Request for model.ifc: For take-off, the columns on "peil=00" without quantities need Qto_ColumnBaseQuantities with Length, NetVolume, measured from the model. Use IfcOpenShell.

First a look at what the model holds.

```python
import ifcopenshell
import ifcopenshell.util.element
import ifcopenshell.util.unit

model = ifcopenshell.open("model.ifc")
print(model.schema)
for unit_type in ("LENGTHUNIT", "AREAUNIT", "VOLUMEUNIT"):
    print(unit_type, ifcopenshell.util.unit.calculate_unit_scale(model, unit_type))
storey = next(s for s in model.by_type("IfcBuildingStorey") if s.Name == "peil=00")
columns = [e for e in ifcopenshell.util.element.get_decomposition(storey) if e.is_a("IfcColumn")]
for e in sorted(columns, key=lambda e: e.id()):
    print(e.id(), e.is_a(), e.Name, list(ifcopenshell.util.element.get_psets(e, qtos_only=True)), sep=" | ")
```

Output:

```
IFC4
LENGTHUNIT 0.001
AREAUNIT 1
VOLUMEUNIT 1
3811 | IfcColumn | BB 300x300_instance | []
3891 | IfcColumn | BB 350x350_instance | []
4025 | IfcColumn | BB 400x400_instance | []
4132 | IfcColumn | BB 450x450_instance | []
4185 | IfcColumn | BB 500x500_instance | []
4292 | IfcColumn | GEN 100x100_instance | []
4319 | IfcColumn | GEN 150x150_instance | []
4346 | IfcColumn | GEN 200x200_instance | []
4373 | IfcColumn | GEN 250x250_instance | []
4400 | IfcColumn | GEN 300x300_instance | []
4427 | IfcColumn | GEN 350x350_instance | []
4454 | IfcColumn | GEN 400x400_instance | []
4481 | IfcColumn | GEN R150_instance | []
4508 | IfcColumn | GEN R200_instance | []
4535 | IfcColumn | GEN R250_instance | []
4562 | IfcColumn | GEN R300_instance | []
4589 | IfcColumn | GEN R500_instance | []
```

```python
import ifcopenshell
import ifcopenshell.api.pset
import ifcopenshell.geom
import ifcopenshell.util.element
import ifcopenshell.util.shape
import ifcopenshell.util.unit

model = ifcopenshell.open("model.ifc")
unit_scale = ifcopenshell.util.unit.calculate_unit_scale(model)
volume_scale = ifcopenshell.util.unit.calculate_unit_scale(model, "VOLUMEUNIT")
settings = ifcopenshell.geom.settings()

storey = next(s for s in model.by_type("IfcBuildingStorey") if s.Name == "peil=00")
columns = [e for e in ifcopenshell.util.element.get_decomposition(storey) if e.is_a("IfcColumn")]

for e in sorted(columns, key=lambda e: e.id()):
    if ifcopenshell.util.element.get_psets(e, qtos_only=True, should_inherit=False):
        continue
    # Geometry comes back in metres, in the element's own axes.
    shape = ifcopenshell.geom.create_shape(settings, e)
    values = {
        "Length": ifcopenshell.util.shape.get_z(shape.geometry) / unit_scale,
        "NetVolume": ifcopenshell.util.shape.get_volume(shape.geometry) / volume_scale,
    }
    qto = ifcopenshell.api.pset.add_qto(model, product=e, name="Qto_ColumnBaseQuantities")
    ifcopenshell.api.pset.edit_qto(model, qto=qto, properties=values)
    print(e.id(), {k: round(v, 3) for k, v in values.items()})

model.write("model_rev.ifc")
```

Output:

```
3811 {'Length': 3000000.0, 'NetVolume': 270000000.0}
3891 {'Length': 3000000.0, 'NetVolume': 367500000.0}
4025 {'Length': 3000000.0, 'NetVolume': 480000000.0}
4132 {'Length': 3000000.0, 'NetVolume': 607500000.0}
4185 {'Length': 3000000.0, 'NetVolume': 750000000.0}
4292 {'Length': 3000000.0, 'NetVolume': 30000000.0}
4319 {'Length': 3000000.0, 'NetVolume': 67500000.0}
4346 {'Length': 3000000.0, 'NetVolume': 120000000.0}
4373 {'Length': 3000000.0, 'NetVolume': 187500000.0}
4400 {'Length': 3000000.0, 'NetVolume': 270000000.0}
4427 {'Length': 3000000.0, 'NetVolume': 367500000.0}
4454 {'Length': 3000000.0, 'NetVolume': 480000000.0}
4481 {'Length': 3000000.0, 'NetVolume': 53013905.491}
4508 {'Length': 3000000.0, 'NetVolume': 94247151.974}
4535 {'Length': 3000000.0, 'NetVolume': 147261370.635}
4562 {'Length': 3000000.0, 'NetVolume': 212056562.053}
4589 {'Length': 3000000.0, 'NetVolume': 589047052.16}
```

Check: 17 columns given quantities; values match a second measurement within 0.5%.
